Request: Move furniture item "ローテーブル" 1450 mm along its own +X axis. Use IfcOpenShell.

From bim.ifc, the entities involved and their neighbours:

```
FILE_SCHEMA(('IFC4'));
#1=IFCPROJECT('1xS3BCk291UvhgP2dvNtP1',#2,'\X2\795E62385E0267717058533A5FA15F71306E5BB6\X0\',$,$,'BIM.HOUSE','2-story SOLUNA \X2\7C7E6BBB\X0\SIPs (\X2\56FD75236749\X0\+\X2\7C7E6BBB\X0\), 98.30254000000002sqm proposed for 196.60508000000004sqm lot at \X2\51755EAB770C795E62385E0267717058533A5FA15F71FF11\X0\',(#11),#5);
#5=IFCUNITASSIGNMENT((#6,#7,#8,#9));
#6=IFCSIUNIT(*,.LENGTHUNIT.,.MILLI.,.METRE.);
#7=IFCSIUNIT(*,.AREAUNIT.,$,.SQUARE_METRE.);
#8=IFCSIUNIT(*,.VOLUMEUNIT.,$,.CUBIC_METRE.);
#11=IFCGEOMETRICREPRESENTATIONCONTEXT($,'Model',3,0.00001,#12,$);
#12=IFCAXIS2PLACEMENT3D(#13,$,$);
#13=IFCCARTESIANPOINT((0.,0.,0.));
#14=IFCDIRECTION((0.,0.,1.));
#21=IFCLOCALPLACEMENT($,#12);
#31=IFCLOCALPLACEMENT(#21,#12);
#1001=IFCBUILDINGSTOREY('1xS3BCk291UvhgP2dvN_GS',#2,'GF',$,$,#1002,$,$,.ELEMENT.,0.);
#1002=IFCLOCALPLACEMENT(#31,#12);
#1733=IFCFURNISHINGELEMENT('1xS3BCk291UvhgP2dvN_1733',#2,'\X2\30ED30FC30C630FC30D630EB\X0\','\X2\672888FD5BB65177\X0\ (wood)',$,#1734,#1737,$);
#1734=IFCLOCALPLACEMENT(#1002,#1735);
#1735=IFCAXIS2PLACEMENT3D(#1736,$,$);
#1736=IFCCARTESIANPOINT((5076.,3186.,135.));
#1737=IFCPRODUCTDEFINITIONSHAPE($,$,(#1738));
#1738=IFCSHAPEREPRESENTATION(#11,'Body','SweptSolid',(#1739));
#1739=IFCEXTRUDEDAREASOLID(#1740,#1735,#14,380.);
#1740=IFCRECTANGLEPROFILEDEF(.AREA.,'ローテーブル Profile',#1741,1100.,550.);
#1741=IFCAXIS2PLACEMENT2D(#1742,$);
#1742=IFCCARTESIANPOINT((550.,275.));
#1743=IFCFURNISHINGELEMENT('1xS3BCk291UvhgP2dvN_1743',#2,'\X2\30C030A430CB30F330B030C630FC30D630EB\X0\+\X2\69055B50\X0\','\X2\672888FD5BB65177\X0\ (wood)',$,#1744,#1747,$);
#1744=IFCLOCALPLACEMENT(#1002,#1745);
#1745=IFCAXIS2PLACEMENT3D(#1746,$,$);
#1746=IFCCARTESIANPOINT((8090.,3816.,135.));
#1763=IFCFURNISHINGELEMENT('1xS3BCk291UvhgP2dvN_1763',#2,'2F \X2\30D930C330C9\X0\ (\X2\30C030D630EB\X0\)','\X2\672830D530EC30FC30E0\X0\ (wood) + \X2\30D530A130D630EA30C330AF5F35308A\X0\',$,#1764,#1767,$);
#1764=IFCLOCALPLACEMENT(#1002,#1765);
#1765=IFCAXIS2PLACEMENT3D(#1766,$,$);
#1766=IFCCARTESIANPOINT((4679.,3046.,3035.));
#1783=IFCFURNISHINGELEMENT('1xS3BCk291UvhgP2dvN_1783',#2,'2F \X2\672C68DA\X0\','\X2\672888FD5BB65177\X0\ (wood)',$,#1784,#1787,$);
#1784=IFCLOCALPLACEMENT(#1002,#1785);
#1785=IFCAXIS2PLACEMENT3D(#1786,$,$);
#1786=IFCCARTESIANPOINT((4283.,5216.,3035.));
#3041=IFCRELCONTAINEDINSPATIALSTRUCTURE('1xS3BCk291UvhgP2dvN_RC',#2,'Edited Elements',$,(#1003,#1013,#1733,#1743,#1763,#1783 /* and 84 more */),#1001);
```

```python
import ifcopenshell
import ifcopenshell.api.geometry
import ifcopenshell.util.placement
import ifcopenshell.util.unit

model = ifcopenshell.open("bim.ifc")
unit_scale = ifcopenshell.util.unit.calculate_unit_scale(model)

item = model.by_guid("1xS3BCk291UvhgP2dvN_1733")
matrix = ifcopenshell.util.placement.get_local_placement(item.ObjectPlacement)
matrix[:3, 3] += matrix[:3, 0] * 1.45 / unit_scale
ifcopenshell.api.geometry.edit_object_placement(model, product=item, matrix=matrix, is_si=False)

print(ifcopenshell.util.placement.get_local_placement(item.ObjectPlacement).round(3) + 0.0)

model.write("bim_v2.ifc")
```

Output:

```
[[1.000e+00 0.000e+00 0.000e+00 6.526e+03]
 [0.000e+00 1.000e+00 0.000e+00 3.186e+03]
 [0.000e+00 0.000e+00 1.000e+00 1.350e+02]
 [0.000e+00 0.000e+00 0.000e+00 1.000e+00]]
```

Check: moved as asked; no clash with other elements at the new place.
